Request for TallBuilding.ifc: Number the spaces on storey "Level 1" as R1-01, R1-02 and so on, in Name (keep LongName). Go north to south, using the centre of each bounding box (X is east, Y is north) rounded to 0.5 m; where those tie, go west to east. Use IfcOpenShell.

First a look at what the model holds.

```python
import ifcopenshell
import ifcopenshell.util.element
import ifcopenshell.util.placement

model = ifcopenshell.open("TallBuilding.ifc")
print(model.schema)
storey = next(s for s in model.by_type("IfcBuildingStorey") if s.Name == "Level 1")
spaces = [e for e in ifcopenshell.util.element.get_decomposition(storey) if e.is_a("IfcSpace")]
for e in sorted(spaces, key=lambda e: e.id()):
    origin = ifcopenshell.util.placement.get_local_placement(e.ObjectPlacement)[:3, 3]
    print(e.id(), e.Name, e.LongName, origin.round(2) + 0.0, sep=" | ")
```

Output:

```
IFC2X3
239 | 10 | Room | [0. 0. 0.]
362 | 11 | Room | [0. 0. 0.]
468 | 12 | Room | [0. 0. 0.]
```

```python
import ifcopenshell
import ifcopenshell.geom
import ifcopenshell.util.element
import ifcopenshell.util.shape

model = ifcopenshell.open("TallBuilding.ifc")
settings = ifcopenshell.geom.settings()
settings.set("use-world-coords", True)


def centre(element):
    shape = ifcopenshell.geom.create_shape(settings, element)
    return ifcopenshell.util.shape.get_bbox_centroid(shape.geometry)


storey = next(s for s in model.by_type("IfcBuildingStorey") if s.Name == "Level 1")
spaces = [e for e in ifcopenshell.util.element.get_decomposition(storey) if e.is_a("IfcSpace")]

# Insertion points can sit at a corner or the storey origin, so sort by the geometry (in metres).
centres = {e: centre(e) for e in spaces}
spaces.sort(key=lambda e: (-round(centres[e][1] / 0.5), centres[e][0]))

for i, e in enumerate(spaces, start=1):
    number = f"R1-{i:02d}"
    e.Name = number
    print(e.id(), number)

model.write("TallBuilding_updated.ifc")
```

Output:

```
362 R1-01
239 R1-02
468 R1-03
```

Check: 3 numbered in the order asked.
